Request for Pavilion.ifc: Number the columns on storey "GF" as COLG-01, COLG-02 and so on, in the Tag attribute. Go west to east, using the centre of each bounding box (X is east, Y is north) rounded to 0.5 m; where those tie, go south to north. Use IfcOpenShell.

First a look at what the model holds.

```python
import ifcopenshell
import ifcopenshell.util.element
import ifcopenshell.util.placement

model = ifcopenshell.open("Pavilion.ifc")
print(model.schema)
storey = next(s for s in model.by_type("IfcBuildingStorey") if s.Name == "GF")
columns = [e for e in ifcopenshell.util.element.get_decomposition(storey) if e.is_a("IfcColumn")]
for e in sorted(columns, key=lambda e: e.id()):
    origin = ifcopenshell.util.placement.get_local_placement(e.ObjectPlacement)[:3, 3]
    print(e.id(), e.Tag, e.Name, origin.round(2) + 0.0, sep=" | ")
```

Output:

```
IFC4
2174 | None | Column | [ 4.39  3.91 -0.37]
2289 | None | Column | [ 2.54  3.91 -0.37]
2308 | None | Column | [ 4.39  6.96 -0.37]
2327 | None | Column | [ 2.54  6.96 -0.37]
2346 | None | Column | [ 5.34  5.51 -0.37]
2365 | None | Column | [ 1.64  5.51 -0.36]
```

```python
import ifcopenshell
import ifcopenshell.geom
import ifcopenshell.util.element
import ifcopenshell.util.shape

model = ifcopenshell.open("Pavilion.ifc")
settings = ifcopenshell.geom.settings()
settings.set("use-world-coords", True)


def centre(element):
    shape = ifcopenshell.geom.create_shape(settings, element)
    return ifcopenshell.util.shape.get_bbox_centroid(shape.geometry)


storey = next(s for s in model.by_type("IfcBuildingStorey") if s.Name == "GF")
columns = [e for e in ifcopenshell.util.element.get_decomposition(storey) if e.is_a("IfcColumn")]

# Insertion points can sit at a corner or the storey origin, so sort by the geometry (in metres).
centres = {e: centre(e) for e in columns}
columns.sort(key=lambda e: (round(centres[e][0] / 0.5), centres[e][1]))

for i, e in enumerate(columns, start=1):
    number = f"COLG-{i:02d}"
    e.Tag = number
    print(e.id(), number)

model.write("Pavilion_edited.ifc")
```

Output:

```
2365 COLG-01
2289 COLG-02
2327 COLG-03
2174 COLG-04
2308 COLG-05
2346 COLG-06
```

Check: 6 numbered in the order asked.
